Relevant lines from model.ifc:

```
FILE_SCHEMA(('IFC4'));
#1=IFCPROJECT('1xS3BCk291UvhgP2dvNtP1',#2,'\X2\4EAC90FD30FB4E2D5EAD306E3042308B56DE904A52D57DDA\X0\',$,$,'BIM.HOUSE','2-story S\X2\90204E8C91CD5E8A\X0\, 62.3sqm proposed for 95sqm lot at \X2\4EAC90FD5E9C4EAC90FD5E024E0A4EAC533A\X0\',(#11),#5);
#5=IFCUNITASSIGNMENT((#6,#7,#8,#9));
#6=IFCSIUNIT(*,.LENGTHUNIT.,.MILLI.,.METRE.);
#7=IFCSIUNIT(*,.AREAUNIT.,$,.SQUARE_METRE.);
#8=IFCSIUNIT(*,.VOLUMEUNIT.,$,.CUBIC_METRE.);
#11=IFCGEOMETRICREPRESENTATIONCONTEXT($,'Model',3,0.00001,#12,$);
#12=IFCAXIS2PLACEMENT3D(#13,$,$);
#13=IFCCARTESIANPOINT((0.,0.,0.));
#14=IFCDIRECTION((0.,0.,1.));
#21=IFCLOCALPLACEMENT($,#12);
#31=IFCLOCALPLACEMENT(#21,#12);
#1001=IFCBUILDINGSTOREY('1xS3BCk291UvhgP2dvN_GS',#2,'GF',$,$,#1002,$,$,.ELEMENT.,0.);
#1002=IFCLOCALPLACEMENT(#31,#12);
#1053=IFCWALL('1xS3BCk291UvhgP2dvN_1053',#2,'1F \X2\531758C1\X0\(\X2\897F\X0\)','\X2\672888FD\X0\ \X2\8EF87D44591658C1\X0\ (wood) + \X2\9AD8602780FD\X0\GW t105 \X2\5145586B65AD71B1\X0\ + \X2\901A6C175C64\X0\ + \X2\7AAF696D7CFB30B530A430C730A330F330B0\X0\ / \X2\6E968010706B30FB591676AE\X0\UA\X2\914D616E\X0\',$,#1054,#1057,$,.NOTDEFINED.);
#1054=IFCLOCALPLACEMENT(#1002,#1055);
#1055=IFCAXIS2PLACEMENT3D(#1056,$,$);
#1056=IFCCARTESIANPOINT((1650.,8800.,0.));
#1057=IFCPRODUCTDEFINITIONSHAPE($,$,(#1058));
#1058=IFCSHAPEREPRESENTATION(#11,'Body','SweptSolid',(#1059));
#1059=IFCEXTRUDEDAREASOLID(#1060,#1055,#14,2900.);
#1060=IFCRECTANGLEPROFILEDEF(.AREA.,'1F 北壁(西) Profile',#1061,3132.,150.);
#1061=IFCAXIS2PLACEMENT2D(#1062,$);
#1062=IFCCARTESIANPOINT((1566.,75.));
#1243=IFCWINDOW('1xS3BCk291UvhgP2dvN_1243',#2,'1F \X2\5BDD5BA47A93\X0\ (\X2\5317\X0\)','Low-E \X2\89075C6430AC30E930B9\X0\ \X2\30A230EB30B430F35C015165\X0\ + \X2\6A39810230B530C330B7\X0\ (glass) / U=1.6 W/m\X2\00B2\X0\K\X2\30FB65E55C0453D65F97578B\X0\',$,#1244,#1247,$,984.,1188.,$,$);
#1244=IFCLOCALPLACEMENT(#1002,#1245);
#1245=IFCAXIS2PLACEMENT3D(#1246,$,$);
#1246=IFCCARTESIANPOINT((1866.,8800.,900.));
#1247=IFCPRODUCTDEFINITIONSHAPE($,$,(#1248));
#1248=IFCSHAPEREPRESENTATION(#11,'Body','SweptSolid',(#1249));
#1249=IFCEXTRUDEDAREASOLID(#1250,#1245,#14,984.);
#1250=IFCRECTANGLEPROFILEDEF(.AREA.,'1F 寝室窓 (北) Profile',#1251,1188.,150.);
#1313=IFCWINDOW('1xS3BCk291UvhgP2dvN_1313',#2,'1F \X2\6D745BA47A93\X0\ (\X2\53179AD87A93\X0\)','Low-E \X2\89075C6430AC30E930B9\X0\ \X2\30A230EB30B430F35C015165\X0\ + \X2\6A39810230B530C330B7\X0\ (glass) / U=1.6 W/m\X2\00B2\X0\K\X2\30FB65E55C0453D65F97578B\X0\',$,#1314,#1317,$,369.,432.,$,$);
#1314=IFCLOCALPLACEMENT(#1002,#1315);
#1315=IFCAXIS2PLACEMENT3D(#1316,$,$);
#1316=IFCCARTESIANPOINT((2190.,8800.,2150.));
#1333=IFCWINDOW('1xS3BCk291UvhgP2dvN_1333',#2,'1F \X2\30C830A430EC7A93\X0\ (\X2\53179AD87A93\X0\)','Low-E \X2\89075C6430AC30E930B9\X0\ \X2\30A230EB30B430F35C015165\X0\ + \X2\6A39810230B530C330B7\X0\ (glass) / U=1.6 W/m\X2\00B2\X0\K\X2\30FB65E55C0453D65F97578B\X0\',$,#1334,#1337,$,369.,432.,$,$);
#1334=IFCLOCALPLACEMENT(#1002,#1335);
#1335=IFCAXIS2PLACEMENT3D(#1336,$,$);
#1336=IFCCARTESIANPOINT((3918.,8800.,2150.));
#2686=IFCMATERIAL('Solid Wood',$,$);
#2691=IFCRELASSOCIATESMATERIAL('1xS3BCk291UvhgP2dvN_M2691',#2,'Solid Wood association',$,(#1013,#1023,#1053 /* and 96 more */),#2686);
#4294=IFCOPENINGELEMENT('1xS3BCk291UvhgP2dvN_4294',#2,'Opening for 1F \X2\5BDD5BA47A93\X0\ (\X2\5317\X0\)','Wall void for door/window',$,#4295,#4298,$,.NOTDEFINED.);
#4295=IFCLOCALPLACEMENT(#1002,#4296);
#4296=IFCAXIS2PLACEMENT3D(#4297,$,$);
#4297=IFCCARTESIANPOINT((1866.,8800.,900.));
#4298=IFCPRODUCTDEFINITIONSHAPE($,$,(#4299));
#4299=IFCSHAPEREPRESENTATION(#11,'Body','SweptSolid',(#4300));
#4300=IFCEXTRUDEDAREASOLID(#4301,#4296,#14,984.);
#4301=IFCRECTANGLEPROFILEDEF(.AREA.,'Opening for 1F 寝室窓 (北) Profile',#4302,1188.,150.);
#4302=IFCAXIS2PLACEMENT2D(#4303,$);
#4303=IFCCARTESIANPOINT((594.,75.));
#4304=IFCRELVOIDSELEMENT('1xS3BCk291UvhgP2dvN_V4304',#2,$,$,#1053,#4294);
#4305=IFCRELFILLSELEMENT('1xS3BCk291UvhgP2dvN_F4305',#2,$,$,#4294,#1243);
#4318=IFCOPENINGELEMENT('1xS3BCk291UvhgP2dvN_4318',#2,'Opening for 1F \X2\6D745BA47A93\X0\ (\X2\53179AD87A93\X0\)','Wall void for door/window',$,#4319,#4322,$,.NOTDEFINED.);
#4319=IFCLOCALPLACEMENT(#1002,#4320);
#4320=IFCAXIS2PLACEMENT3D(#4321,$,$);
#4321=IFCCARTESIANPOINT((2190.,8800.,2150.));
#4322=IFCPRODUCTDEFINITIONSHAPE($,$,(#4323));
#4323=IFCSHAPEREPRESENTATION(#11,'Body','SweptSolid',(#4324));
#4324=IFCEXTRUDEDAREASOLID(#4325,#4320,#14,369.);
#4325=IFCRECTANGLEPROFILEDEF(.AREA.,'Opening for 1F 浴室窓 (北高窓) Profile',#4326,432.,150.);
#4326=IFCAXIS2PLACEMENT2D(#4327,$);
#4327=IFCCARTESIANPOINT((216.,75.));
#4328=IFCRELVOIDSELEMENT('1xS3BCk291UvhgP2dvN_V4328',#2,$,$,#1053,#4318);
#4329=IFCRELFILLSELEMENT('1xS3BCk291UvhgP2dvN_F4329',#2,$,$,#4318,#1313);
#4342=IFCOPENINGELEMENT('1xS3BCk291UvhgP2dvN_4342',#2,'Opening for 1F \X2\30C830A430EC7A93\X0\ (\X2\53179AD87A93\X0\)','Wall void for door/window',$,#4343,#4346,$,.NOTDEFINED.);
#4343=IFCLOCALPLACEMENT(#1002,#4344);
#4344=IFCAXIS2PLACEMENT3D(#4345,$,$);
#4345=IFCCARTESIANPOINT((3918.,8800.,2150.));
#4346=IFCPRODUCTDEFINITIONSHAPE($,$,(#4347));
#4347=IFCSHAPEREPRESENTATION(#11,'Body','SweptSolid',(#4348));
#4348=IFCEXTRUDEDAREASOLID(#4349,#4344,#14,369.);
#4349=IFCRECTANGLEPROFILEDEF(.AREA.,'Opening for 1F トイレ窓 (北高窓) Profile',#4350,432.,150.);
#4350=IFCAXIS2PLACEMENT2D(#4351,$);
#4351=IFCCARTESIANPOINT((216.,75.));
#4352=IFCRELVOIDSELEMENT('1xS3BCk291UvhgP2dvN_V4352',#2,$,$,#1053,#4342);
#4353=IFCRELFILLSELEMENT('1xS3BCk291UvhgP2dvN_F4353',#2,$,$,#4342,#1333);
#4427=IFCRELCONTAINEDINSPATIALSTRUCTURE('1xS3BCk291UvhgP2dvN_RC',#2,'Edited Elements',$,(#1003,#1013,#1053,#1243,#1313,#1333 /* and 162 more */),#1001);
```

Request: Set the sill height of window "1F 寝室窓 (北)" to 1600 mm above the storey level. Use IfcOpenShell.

```python
import numpy as np
import ifcopenshell
import ifcopenshell.api.geometry
import ifcopenshell.geom
import ifcopenshell.util.element
import ifcopenshell.util.placement
import ifcopenshell.util.shape
import ifcopenshell.util.unit

model = ifcopenshell.open("model.ifc")
unit_scale = ifcopenshell.util.unit.calculate_unit_scale(model)

window = model.by_id(1243)
opening = window.FillsVoids[0].RelatingOpeningElement
storey = ifcopenshell.util.element.get_container(window, ifc_class="IfcBuildingStorey")
level = ifcopenshell.util.placement.get_local_placement(storey.ObjectPlacement)[2, 3]

# The opening's origin need not be at the sill, so measure its lowest point.
shape = ifcopenshell.geom.create_shape(ifcopenshell.geom.settings(), opening)
bottom = ifcopenshell.util.shape.get_shape_bottom_elevation(shape, shape.geometry) / unit_scale
dz = level + 1600.0 - bottom

shift = np.array([0.0, 0.0, dz])
# The window is not placed relative to its opening, so move both.
for product in (opening, window):
    matrix = ifcopenshell.util.placement.get_local_placement(product.ObjectPlacement)
    matrix[:3, 3] += shift
    ifcopenshell.api.geometry.edit_object_placement(model, product=product, matrix=matrix, is_si=False)

print(f"moved by {dz * unit_scale:+.3f} m")

model.write("model_rev.ifc")
```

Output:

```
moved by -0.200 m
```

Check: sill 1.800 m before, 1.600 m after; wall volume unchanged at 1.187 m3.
